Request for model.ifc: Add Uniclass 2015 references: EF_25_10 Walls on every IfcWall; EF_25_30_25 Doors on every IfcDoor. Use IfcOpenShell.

First a look at what the model holds.

```python
import ifcopenshell

model = ifcopenshell.open("model.ifc")
print(model.schema)
print("classifications:", [c.Name for c in model.by_type("IfcClassification")])
for ifc_class in ("IfcDoor", "IfcRoof", "IfcStair", "IfcWall", "IfcWindow"):
    print(ifc_class, len(model.by_type(ifc_class)))
```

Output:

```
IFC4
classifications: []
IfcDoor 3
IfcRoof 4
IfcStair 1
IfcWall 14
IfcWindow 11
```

```python
import ifcopenshell
import ifcopenshell.api.classification

model = ifcopenshell.open("model.ifc")

system = ifcopenshell.api.classification.add_classification(model, classification="Uniclass 2015")

codes = {
    "IfcWall": ("EF_25_10", "Walls"),
    "IfcDoor": ("EF_25_30_25", "Doors"),
}
for ifc_class, (code, name) in codes.items():
    products = model.by_type(ifc_class)
    ifcopenshell.api.classification.add_reference(
        model, products=products, classification=system, identification=code, name=name
    )
    print(code, len(products))

model.write("model_updated.ifc")
```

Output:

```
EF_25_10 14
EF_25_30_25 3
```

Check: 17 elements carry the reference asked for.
